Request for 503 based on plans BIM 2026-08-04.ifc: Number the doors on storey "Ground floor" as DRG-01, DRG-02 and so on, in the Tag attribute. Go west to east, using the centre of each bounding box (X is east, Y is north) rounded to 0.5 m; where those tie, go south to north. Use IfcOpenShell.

First a look at what the model holds.

```python
import ifcopenshell
import ifcopenshell.util.element
import ifcopenshell.util.placement

model = ifcopenshell.open("503 based on plans BIM 2026-08-04.ifc")
print(model.schema)
storey = next(s for s in model.by_type("IfcBuildingStorey") if s.Name == "Ground floor")
doors = [e for e in ifcopenshell.util.element.get_decomposition(storey) if e.is_a("IfcDoor")]
for e in sorted(doors, key=lambda e: e.id()):
    origin = ifcopenshell.util.placement.get_local_placement(e.ObjectPlacement)[:3, 3]
    print(e.id(), e.Tag, e.Name, origin.round(2) + 0.0, sep=" | ")
```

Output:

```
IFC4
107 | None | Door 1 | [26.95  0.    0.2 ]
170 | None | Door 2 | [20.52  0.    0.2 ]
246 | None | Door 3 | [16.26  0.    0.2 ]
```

```python
import ifcopenshell
import ifcopenshell.geom
import ifcopenshell.util.element
import ifcopenshell.util.shape

model = ifcopenshell.open("503 based on plans BIM 2026-08-04.ifc")
settings = ifcopenshell.geom.settings()
settings.set("use-world-coords", True)


def centre(element):
    shape = ifcopenshell.geom.create_shape(settings, element)
    return ifcopenshell.util.shape.get_bbox_centroid(shape.geometry)


storey = next(s for s in model.by_type("IfcBuildingStorey") if s.Name == "Ground floor")
doors = [e for e in ifcopenshell.util.element.get_decomposition(storey) if e.is_a("IfcDoor")]

# Insertion points can sit at a corner or the storey origin, so sort by the geometry (in metres).
centres = {e: centre(e) for e in doors}
doors.sort(key=lambda e: (round(centres[e][0] / 0.5), centres[e][1]))

for i, e in enumerate(doors, start=1):
    number = f"DRG-{i:02d}"
    e.Tag = number
    print(e.id(), number)

model.write("503 based on plans BIM 2026-08-04_rev.ifc")
```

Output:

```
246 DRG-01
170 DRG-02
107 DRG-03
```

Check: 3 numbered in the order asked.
